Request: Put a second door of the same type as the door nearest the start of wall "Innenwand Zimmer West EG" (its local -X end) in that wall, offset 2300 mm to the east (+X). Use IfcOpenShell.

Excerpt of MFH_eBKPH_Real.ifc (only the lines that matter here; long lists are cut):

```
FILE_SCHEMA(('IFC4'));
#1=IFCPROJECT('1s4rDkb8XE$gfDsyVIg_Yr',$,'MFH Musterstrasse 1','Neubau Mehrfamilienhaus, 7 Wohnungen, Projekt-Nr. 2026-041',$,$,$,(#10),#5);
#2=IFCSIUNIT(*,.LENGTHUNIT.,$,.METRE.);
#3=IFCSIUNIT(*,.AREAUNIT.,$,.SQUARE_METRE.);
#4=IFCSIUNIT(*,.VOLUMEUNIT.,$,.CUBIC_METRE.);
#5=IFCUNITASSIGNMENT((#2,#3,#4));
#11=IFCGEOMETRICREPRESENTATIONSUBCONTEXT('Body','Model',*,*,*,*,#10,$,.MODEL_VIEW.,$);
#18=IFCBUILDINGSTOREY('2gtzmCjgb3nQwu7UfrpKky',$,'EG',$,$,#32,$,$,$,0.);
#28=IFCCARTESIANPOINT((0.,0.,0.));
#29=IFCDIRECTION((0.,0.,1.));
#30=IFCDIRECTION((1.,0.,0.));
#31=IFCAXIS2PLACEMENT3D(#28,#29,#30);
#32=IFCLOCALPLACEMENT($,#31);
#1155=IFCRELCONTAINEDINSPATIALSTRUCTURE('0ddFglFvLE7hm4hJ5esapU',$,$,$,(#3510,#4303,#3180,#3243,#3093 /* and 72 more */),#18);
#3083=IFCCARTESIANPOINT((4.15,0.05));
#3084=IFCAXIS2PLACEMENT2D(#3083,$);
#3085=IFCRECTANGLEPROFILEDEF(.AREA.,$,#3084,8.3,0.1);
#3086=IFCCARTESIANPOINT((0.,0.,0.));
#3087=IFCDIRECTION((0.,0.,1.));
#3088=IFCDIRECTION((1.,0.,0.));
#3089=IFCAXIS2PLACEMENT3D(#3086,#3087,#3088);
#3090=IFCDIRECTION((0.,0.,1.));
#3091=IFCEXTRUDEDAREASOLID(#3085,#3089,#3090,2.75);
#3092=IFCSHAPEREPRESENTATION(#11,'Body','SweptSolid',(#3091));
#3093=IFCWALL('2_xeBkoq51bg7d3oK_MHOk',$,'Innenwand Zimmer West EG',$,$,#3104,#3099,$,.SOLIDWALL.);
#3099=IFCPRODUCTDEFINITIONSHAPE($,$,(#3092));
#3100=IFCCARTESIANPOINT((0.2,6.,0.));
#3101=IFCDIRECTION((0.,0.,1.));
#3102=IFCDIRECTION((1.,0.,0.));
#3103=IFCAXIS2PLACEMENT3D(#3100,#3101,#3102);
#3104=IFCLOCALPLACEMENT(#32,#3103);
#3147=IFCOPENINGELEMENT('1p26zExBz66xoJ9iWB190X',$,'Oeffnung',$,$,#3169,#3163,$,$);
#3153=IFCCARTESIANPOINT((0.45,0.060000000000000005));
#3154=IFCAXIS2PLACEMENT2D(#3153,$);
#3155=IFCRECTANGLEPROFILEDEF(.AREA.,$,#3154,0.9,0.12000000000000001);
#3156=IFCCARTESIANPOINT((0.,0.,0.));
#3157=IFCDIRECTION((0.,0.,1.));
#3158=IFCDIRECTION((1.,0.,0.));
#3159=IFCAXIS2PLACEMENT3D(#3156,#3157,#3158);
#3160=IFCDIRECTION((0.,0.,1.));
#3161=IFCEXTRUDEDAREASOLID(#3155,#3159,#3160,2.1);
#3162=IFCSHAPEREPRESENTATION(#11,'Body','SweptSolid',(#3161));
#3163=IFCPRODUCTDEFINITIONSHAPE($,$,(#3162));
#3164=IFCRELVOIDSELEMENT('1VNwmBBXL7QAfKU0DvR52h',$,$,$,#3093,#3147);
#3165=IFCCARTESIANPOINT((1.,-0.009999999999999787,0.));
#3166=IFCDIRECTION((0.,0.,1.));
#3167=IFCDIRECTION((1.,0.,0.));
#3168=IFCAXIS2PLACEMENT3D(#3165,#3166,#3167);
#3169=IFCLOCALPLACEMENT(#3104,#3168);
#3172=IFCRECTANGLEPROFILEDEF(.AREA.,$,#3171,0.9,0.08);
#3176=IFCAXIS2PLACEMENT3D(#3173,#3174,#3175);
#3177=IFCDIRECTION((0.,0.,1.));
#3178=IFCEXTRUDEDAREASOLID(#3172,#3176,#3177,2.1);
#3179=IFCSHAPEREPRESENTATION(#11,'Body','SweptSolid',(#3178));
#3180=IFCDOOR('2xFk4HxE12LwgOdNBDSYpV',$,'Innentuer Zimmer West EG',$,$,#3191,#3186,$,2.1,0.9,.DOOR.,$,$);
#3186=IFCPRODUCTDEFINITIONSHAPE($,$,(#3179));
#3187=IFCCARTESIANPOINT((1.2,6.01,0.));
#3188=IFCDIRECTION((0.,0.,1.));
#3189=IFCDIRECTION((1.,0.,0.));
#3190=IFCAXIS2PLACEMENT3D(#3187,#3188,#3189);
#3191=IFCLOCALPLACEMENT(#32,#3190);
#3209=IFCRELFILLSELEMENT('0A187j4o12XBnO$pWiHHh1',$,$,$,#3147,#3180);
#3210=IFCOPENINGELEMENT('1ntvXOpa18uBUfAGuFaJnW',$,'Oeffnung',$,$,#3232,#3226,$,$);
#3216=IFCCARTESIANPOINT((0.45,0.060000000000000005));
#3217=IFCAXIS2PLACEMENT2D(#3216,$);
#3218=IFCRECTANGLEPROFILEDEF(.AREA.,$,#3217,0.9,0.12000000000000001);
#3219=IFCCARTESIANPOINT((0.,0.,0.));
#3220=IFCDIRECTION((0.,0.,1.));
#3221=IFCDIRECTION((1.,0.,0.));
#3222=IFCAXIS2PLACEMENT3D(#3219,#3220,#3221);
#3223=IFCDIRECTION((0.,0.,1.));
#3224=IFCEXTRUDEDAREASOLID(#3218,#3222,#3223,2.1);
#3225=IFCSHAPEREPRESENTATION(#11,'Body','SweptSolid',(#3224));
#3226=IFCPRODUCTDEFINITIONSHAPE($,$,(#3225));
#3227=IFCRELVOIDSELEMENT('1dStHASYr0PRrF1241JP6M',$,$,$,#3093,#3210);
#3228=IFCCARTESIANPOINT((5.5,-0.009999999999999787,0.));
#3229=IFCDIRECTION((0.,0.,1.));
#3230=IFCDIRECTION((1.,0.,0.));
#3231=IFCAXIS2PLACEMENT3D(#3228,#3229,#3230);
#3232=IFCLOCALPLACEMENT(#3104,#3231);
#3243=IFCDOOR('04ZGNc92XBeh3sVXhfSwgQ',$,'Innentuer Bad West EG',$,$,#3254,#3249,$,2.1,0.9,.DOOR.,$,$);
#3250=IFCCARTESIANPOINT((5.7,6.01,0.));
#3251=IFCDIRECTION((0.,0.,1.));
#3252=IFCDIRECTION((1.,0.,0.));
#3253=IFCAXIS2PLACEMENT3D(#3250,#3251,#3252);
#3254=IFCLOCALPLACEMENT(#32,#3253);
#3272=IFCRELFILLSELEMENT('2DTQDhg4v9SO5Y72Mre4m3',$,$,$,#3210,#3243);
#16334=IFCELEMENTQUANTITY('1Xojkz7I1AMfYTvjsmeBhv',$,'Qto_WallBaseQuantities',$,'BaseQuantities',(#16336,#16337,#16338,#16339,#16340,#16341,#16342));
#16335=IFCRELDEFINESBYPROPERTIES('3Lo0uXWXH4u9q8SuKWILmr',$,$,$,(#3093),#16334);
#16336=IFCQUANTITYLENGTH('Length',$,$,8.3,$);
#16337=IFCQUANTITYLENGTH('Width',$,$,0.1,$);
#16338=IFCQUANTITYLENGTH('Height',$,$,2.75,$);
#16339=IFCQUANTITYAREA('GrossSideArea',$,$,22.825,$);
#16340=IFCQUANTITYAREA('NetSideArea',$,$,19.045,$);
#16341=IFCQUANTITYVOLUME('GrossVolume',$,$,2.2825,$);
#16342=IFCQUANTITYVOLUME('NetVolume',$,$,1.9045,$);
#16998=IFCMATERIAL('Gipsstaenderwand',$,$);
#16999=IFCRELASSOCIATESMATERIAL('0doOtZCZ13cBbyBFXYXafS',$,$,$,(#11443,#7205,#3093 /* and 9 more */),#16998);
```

```python
import ifcopenshell
import ifcopenshell.api.feature
import ifcopenshell.api.geometry
import ifcopenshell.api.pset
import ifcopenshell.api.root
import ifcopenshell.geom
import ifcopenshell.util.element
import ifcopenshell.util.placement
import ifcopenshell.util.shape
import ifcopenshell.util.unit

model = ifcopenshell.open("MFH_eBKPH_Real.ifc")
area_scale = ifcopenshell.util.unit.calculate_unit_scale(model, "AREAUNIT")
volume_scale = ifcopenshell.util.unit.calculate_unit_scale(model, "VOLUMEUNIT")
settings = ifcopenshell.geom.settings()


def volume(element):
    """Net volume in cubic metres, openings subtracted."""
    shape = ifcopenshell.geom.create_shape(settings, element)
    return ifcopenshell.util.shape.get_volume(shape.geometry)


door = model.by_guid("2xFk4HxE12LwgOdNBDSYpV")
opening = door.FillsVoids[0].RelatingOpeningElement
wall = opening.VoidsElements[0].RelatingBuildingElement
before = volume(wall)
shift = ifcopenshell.util.placement.get_local_placement(wall.ObjectPlacement)[:3, 0] * 2.3

# copy_class copies the void relationship, type, container and properties, but no geometry.
new_opening = ifcopenshell.api.root.copy_class(model, product=opening)
new_opening.Representation = ifcopenshell.util.element.copy_deep(
    model, opening.Representation, exclude=["IfcGeometricRepresentationContext", "IfcRepresentationMap"]
)
new_door = ifcopenshell.api.root.copy_class(model, product=door)
new_door.Representation = ifcopenshell.util.element.copy_deep(
    model, door.Representation, exclude=["IfcGeometricRepresentationContext", "IfcRepresentationMap"]
)
ifcopenshell.api.feature.add_filling(model, opening=new_opening, element=new_door)

for old, new in ((opening, new_opening), (door, new_door)):
    matrix = ifcopenshell.util.placement.get_local_placement(old.ObjectPlacement)
    matrix[:3, 3] += shift
    ifcopenshell.api.geometry.edit_object_placement(model, product=new, matrix=matrix, is_si=False)

after = volume(wall)
thickness = 0.1  # wall thickness in metres

# Update the wall's stored quantities.
qto = model.by_id(ifcopenshell.util.element.get_pset(wall, "Qto_WallBaseQuantities", should_inherit=False)["id"])
ifcopenshell.api.pset.edit_qto(model, qto=qto, properties={
    "NetSideArea": after / thickness / area_scale,
    "NetVolume": after / volume_scale,
})

print(f"wall volume {before:.3f} -> {after:.3f} m3")

model.write("MFH_eBKPH_Real_edited.ifc")
```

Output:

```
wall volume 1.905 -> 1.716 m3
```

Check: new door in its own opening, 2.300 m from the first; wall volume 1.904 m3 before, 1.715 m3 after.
